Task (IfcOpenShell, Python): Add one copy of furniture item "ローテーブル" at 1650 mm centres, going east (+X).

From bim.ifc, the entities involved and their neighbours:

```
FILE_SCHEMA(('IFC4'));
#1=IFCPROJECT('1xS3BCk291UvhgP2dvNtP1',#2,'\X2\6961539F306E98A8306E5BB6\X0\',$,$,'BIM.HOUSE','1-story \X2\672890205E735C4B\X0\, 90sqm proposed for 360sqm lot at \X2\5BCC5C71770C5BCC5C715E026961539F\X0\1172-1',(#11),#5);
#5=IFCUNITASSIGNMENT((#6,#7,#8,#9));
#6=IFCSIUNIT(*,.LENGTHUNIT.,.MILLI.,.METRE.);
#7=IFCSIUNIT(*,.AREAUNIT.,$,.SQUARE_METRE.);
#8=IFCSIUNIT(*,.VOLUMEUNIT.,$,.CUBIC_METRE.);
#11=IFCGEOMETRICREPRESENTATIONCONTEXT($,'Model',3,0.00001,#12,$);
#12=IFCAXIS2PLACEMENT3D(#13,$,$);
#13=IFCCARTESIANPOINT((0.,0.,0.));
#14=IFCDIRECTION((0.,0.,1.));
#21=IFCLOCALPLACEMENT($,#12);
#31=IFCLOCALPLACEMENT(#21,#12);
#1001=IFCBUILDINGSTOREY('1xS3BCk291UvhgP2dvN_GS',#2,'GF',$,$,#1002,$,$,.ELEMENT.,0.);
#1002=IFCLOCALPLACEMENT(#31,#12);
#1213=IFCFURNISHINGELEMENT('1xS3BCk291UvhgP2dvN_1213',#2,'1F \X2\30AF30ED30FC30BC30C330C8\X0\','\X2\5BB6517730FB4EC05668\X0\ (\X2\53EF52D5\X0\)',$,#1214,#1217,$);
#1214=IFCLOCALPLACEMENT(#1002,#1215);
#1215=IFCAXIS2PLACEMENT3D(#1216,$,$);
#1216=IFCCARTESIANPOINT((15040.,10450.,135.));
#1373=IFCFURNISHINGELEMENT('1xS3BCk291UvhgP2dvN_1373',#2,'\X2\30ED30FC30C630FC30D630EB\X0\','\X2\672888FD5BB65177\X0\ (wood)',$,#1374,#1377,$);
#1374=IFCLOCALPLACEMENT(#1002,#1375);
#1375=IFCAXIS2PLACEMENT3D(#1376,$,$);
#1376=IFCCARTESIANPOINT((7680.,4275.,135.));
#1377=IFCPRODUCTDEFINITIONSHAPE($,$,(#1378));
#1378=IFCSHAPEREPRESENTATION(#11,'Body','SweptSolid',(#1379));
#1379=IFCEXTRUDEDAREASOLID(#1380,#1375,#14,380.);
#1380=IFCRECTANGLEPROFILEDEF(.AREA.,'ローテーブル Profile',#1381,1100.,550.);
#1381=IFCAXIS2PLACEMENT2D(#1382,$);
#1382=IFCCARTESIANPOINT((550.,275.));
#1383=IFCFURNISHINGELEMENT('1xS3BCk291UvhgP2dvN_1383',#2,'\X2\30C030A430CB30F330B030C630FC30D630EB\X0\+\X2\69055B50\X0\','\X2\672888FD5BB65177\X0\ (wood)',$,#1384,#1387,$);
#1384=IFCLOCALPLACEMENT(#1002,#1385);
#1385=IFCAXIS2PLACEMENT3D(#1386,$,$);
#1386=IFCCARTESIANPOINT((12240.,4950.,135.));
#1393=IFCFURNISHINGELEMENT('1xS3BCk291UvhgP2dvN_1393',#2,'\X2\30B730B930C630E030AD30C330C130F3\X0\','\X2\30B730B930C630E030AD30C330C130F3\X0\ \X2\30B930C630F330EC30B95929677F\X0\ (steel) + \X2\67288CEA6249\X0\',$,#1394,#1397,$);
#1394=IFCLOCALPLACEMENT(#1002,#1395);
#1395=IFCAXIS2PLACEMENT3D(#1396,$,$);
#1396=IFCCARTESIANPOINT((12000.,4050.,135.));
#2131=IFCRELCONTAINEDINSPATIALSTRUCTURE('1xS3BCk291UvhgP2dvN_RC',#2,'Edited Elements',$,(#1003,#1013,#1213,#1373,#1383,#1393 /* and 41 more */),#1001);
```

```python
import numpy as np
import ifcopenshell
import ifcopenshell.api.geometry
import ifcopenshell.api.root
import ifcopenshell.util.element
import ifcopenshell.util.placement

model = ifcopenshell.open("bim.ifc")


def reuse_history(source, copy):
    """copy_class also copies each property set's owner history, people and application; keep the originals."""
    for rel in copy.IsDefinedBy:
        if rel.is_a("IfcRelDefinesByProperties") and (history := rel.RelatingPropertyDefinition.OwnerHistory):
            rel.RelatingPropertyDefinition.OwnerHistory = source.OwnerHistory
            ifcopenshell.util.element.remove_deep2(model, history)


source = model.by_guid("1xS3BCk291UvhgP2dvN_1373")
base = ifcopenshell.util.placement.get_local_placement(source.ObjectPlacement)
step = np.array([1.0, 0.0, 0.0]) * 1650.0

for i in range(1, 2):
    copy = ifcopenshell.api.root.copy_class(model, product=source)
    copy.Representation = ifcopenshell.util.element.copy_deep(
        model, source.Representation, exclude=["IfcGeometricRepresentationContext", "IfcRepresentationMap"]
    )
    reuse_history(source, copy)
    matrix = base.copy()
    matrix[:3, 3] += i * step
    print("added at", matrix[:3, 3].round(3) + 0.0)
    ifcopenshell.api.geometry.edit_object_placement(model, product=copy, matrix=matrix, is_si=False)

model.write("bim_v2.ifc")
```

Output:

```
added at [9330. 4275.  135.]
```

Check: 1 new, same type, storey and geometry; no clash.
